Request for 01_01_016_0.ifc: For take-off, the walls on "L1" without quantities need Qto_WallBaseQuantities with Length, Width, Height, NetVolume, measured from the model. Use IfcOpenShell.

First a look at what the model holds.

```python
import ifcopenshell
import ifcopenshell.util.element
import ifcopenshell.util.unit

model = ifcopenshell.open("01_01_016_0.ifc")
print(model.schema)
for unit_type in ("LENGTHUNIT", "AREAUNIT", "VOLUMEUNIT"):
    print(unit_type, ifcopenshell.util.unit.calculate_unit_scale(model, unit_type))
storey = next(s for s in model.by_type("IfcBuildingStorey") if s.Name == "L1")
walls = [e for e in ifcopenshell.util.element.get_decomposition(storey) if e.is_a("IfcWall")]
for e in sorted(walls, key=lambda e: e.id()):
    print(e.id(), e.is_a(), e.Name, list(ifcopenshell.util.element.get_psets(e, qtos_only=True)), sep=" | ")
```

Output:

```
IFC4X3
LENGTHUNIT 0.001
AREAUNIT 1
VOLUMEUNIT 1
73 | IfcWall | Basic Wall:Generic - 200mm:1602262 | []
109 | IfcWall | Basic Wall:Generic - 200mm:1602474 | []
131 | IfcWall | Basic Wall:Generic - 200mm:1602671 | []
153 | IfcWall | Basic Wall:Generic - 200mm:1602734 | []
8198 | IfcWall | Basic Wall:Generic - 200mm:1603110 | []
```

```python
import ifcopenshell
import ifcopenshell.api.pset
import ifcopenshell.geom
import ifcopenshell.util.element
import ifcopenshell.util.shape
import ifcopenshell.util.unit

model = ifcopenshell.open("01_01_016_0.ifc")
unit_scale = ifcopenshell.util.unit.calculate_unit_scale(model)
volume_scale = ifcopenshell.util.unit.calculate_unit_scale(model, "VOLUMEUNIT")
settings = ifcopenshell.geom.settings()

storey = next(s for s in model.by_type("IfcBuildingStorey") if s.Name == "L1")
walls = [e for e in ifcopenshell.util.element.get_decomposition(storey) if e.is_a("IfcWall")]

for e in sorted(walls, key=lambda e: e.id()):
    if ifcopenshell.util.element.get_psets(e, qtos_only=True, should_inherit=False):
        continue
    # Geometry comes back in metres, in the element's own axes.
    shape = ifcopenshell.geom.create_shape(settings, e)
    values = {
        "Length": ifcopenshell.util.shape.get_x(shape.geometry) / unit_scale,
        "Width": ifcopenshell.util.shape.get_y(shape.geometry) / unit_scale,
        "Height": ifcopenshell.util.shape.get_z(shape.geometry) / unit_scale,
        "NetVolume": ifcopenshell.util.shape.get_volume(shape.geometry) / volume_scale,
    }
    qto = ifcopenshell.api.pset.add_qto(model, product=e, name="Qto_WallBaseQuantities")
    ifcopenshell.api.pset.edit_qto(model, qto=qto, properties=values)
    print(e.id(), {k: round(v, 3) for k, v in values.items()})

model.write("01_01_016_0_updated.ifc")
```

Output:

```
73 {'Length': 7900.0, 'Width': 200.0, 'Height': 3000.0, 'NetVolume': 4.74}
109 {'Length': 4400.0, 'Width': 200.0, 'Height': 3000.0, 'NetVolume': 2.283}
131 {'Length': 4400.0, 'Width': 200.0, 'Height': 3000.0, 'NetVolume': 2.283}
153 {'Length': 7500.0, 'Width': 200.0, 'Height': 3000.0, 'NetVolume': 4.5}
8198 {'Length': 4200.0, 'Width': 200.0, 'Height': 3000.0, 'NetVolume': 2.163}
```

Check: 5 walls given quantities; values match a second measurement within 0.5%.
